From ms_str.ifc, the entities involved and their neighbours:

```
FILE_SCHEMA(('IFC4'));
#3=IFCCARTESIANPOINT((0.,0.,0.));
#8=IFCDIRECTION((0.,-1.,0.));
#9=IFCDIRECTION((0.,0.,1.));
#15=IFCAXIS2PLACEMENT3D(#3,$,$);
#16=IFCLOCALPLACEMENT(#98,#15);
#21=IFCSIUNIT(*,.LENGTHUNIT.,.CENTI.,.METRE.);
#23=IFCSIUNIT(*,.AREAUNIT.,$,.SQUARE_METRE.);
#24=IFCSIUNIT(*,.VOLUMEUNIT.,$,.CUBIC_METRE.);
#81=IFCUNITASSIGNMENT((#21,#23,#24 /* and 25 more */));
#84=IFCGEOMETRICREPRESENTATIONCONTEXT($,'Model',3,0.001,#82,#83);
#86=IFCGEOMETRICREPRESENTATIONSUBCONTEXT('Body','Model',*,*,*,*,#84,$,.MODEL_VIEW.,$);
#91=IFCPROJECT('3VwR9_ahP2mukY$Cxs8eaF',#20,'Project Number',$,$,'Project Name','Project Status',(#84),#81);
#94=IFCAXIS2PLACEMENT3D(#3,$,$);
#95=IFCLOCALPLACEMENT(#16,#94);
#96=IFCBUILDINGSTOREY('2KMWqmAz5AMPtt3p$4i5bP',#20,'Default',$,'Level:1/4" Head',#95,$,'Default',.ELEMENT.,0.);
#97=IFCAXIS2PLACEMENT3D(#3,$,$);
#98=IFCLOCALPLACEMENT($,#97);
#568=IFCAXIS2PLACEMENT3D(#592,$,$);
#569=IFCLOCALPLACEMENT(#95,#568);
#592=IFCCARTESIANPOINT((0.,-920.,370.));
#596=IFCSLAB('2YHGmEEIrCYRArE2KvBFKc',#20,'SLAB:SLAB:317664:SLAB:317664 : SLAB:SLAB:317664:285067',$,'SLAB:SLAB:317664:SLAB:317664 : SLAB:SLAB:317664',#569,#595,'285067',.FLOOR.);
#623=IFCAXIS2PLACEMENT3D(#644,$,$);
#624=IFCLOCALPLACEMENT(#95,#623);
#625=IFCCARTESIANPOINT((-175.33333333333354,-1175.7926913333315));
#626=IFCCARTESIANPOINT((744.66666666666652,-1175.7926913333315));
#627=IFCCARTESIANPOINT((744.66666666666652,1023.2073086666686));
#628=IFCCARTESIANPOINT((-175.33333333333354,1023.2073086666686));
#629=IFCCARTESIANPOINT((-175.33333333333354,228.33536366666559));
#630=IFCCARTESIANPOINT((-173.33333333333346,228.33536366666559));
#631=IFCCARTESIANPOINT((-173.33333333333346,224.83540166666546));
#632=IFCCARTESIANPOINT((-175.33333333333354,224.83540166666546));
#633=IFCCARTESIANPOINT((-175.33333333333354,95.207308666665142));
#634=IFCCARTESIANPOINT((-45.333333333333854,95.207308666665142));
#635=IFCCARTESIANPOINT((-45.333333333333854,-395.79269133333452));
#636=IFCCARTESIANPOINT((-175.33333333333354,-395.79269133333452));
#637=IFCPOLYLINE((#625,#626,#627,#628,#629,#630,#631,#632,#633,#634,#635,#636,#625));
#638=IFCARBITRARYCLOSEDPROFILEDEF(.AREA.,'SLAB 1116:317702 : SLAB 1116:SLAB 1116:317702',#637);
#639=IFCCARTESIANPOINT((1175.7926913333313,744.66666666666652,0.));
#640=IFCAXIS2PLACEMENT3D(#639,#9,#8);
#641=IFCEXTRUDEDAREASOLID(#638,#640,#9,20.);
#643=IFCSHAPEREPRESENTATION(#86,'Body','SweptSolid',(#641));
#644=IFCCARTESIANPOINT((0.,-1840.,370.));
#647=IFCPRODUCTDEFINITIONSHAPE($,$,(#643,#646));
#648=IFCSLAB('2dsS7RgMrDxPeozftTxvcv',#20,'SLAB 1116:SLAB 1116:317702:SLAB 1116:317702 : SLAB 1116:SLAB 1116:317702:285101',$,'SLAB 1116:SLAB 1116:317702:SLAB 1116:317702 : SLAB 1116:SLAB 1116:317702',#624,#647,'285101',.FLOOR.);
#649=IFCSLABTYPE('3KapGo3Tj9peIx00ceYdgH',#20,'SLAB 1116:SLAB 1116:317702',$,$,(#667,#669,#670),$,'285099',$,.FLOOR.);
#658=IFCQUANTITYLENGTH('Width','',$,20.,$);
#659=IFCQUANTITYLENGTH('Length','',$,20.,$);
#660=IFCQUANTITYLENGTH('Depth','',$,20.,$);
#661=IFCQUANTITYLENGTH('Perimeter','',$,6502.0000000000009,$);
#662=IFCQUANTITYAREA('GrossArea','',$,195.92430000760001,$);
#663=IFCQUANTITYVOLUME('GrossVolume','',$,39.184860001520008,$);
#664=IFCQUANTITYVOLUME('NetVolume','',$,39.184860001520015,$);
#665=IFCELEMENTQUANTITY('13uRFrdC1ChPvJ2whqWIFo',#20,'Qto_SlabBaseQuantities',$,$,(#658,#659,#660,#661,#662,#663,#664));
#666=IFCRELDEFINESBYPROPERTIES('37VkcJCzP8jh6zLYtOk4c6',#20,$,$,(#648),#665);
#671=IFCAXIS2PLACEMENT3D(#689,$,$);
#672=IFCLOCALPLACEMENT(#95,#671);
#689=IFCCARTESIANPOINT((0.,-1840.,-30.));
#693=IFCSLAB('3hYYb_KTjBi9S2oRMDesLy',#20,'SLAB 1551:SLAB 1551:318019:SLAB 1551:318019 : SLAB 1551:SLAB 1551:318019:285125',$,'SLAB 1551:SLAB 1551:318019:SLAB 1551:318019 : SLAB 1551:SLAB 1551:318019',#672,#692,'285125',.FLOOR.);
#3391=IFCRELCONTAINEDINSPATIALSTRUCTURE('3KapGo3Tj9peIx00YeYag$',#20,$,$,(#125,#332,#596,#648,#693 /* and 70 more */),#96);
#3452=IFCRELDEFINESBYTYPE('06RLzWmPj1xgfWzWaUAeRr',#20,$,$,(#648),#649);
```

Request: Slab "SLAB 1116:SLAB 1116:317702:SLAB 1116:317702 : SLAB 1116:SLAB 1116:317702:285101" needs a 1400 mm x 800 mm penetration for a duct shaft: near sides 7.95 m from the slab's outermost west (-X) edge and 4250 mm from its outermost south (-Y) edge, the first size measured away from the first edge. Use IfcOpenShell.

```python
import numpy as np
import ifcopenshell
import ifcopenshell.api.feature
import ifcopenshell.api.geometry
import ifcopenshell.api.pset
import ifcopenshell.api.root
import ifcopenshell.geom
import ifcopenshell.util.element
import ifcopenshell.util.placement
import ifcopenshell.util.representation
import ifcopenshell.util.shape
import ifcopenshell.util.unit

model = ifcopenshell.open("ms_str.ifc")
unit_scale = ifcopenshell.util.unit.calculate_unit_scale(model)
volume_scale = ifcopenshell.util.unit.calculate_unit_scale(model, "VOLUMEUNIT")
settings = ifcopenshell.geom.settings()


def volume(element):
    """Net volume in cubic metres, openings subtracted."""
    shape = ifcopenshell.geom.create_shape(settings, element)
    return ifcopenshell.util.shape.get_volume(shape.geometry)


slab = model.by_guid("2dsS7RgMrDxPeozftTxvcv")
before = volume(slab)

# Extent in the slab's own axes, in metres. The edges named are its -X and -Y sides.
slab_shape = ifcopenshell.geom.create_shape(settings, slab)
vertices = ifcopenshell.util.shape.get_vertices(slab_shape.geometry)
x_min, y_min, bottom = vertices.min(axis=0)
top = vertices[:, 2].max()

opening = ifcopenshell.api.root.create_entity(model, ifc_class="IfcOpeningElement", name="Duct shaft opening", predefined_type="OPENING")
context = ifcopenshell.util.representation.get_context(model, "Model", "Body", "MODEL_VIEW")
width, depth = 1.4, 0.8
outline = [(0.0, 0.0), (width, 0.0), (width, depth), (0.0, depth), (0.0, 0.0)]
# Overshoot both faces by 50 mm so the cut is clean.
shape = ifcopenshell.api.geometry.add_slab_representation(
    model, context=context, depth=top - bottom + 0.1, polyline=outline
)
ifcopenshell.api.geometry.assign_representation(model, product=opening, representation=shape)

matrix = ifcopenshell.util.placement.get_local_placement(slab.ObjectPlacement)
matrix[:, 3] = matrix @ np.append(np.array([x_min + 7.95, y_min + 4.25, bottom - 0.05]) / unit_scale, 1.0)
ifcopenshell.api.geometry.edit_object_placement(model, product=opening, matrix=matrix, is_si=False)
ifcopenshell.api.feature.add_feature(model, feature=opening, element=slab)

after = volume(slab)

# Update the slab's stored quantities.
qto = model.by_id(ifcopenshell.util.element.get_pset(slab, "Qto_SlabBaseQuantities", should_inherit=False)["id"])
ifcopenshell.api.pset.edit_qto(model, qto=qto, properties={"NetVolume": after / volume_scale})

print(f"slab volume {before:.3f} -> {after:.3f} m3")

model.write("ms_str_rev.ifc")
```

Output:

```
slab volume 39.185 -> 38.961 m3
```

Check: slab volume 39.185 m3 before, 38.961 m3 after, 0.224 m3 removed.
